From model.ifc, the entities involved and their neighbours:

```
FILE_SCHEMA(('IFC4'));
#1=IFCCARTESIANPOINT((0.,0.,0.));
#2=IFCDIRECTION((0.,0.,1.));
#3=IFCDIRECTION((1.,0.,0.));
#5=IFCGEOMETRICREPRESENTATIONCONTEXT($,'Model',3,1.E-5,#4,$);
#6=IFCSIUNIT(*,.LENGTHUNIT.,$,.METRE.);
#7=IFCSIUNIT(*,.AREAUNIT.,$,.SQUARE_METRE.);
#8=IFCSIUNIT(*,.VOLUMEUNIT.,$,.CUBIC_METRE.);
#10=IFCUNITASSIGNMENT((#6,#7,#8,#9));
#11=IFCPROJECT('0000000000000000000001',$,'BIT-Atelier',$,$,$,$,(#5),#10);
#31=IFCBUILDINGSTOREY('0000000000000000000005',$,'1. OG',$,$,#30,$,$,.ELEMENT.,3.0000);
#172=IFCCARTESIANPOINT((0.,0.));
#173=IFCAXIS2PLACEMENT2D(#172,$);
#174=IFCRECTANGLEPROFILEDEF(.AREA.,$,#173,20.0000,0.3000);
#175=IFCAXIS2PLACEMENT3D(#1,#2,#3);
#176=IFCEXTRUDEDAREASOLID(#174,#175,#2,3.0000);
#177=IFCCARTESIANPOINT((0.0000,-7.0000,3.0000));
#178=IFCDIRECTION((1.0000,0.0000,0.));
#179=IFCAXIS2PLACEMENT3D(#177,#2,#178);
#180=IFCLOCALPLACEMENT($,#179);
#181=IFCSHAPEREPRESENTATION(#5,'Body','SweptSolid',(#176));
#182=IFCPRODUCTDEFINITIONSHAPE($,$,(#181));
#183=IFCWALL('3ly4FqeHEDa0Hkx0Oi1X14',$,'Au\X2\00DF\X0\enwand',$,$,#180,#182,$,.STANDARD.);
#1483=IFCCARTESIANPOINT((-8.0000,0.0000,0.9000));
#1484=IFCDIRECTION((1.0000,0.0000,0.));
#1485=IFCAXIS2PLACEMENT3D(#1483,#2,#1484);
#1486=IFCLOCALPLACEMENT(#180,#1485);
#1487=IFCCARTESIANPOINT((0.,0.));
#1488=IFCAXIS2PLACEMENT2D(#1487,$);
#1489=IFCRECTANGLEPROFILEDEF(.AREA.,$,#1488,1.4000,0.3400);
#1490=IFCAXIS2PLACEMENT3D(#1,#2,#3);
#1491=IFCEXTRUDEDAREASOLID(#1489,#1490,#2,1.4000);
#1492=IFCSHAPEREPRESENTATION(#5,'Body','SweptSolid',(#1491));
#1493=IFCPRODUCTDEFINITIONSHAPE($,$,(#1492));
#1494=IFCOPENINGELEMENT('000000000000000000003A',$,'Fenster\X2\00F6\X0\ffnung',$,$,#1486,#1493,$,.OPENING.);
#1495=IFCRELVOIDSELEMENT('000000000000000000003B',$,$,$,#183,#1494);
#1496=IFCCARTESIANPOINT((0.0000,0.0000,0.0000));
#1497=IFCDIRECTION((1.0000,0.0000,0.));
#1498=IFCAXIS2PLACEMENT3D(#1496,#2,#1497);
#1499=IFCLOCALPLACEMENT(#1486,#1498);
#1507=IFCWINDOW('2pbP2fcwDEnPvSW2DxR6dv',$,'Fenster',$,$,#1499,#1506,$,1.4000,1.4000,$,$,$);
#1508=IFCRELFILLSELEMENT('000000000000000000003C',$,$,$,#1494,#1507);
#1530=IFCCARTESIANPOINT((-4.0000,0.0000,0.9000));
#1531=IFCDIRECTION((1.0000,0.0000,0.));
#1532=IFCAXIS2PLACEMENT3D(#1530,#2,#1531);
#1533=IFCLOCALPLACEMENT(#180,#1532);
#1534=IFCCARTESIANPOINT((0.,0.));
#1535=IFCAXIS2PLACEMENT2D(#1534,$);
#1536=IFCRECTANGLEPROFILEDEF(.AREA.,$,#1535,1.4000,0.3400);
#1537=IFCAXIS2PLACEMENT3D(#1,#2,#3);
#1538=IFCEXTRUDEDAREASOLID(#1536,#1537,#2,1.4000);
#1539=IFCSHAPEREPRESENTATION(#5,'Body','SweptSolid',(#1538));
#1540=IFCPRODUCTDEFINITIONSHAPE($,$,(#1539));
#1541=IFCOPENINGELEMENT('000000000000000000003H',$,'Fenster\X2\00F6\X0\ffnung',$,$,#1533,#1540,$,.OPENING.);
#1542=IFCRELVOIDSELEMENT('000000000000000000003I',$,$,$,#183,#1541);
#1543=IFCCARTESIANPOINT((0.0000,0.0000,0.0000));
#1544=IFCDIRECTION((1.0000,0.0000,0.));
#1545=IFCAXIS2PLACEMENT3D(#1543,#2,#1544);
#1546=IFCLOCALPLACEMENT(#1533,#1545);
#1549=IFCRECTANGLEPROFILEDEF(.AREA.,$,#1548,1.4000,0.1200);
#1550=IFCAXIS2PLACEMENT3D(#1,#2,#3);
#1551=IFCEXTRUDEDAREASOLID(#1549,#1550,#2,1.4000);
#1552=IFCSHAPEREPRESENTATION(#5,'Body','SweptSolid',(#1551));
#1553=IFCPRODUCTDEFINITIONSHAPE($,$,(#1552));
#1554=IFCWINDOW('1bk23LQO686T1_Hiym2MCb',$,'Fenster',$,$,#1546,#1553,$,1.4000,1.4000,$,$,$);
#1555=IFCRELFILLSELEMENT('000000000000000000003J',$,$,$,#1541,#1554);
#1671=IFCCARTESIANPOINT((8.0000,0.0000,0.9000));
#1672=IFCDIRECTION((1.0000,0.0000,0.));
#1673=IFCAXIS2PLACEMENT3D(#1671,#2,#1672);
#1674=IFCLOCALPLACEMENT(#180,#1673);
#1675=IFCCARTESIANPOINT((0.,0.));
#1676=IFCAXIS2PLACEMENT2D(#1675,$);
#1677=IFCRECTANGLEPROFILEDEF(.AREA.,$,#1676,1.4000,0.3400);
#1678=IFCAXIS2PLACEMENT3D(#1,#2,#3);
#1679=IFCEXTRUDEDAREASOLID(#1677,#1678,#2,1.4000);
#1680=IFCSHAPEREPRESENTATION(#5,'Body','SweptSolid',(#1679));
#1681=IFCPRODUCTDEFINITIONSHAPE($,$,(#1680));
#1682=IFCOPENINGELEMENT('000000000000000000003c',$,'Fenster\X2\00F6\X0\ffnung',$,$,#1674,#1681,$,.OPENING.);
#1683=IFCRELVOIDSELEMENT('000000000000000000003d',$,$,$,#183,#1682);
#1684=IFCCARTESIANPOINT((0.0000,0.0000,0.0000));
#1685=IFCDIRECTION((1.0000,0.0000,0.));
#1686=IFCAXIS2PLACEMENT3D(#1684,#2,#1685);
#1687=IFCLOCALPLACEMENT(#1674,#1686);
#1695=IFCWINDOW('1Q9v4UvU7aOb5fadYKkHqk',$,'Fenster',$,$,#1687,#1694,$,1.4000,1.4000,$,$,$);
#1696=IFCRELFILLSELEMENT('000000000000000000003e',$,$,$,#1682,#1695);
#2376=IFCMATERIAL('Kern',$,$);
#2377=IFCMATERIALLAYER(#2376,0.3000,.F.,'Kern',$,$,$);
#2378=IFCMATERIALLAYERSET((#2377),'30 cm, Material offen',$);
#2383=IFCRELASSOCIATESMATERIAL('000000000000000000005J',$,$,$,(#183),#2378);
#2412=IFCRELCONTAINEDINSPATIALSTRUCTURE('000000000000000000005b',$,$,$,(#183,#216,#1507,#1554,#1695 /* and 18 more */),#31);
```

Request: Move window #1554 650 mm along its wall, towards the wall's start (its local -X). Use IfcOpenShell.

```python
import ifcopenshell
import ifcopenshell.api.geometry
import ifcopenshell.util.placement

model = ifcopenshell.open("model.ifc")

window = model.by_id(1554)
opening = window.FillsVoids[0].RelatingOpeningElement
wall = opening.VoidsElements[0].RelatingBuildingElement

wall_matrix = ifcopenshell.util.placement.get_local_placement(wall.ObjectPlacement)
shift = wall_matrix[:3, 0] * -0.65
before = ifcopenshell.util.placement.get_local_placement(window.ObjectPlacement)[:3, 3].copy()

# The window is placed relative to its opening, so it follows when the opening moves.
matrix = ifcopenshell.util.placement.get_local_placement(opening.ObjectPlacement)
matrix[:3, 3] += shift
ifcopenshell.api.geometry.edit_object_placement(
    model, product=opening, matrix=matrix, is_si=False, should_transform_children=True
)

after = ifcopenshell.util.placement.get_local_placement(window.ObjectPlacement)[:3, 3]
print("window moved by", (after - before).round(3) + 0.0)

model.write("model_v2.ifc")
```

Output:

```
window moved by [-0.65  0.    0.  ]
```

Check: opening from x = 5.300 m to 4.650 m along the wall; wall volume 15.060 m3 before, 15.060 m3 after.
